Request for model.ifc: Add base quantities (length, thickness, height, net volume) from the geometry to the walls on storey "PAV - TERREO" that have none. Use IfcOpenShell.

First a look at what the model holds.

```python
import ifcopenshell
import ifcopenshell.util.element
import ifcopenshell.util.unit

model = ifcopenshell.open("model.ifc")
print(model.schema)
for unit_type in ("LENGTHUNIT", "AREAUNIT", "VOLUMEUNIT"):
    print(unit_type, ifcopenshell.util.unit.calculate_unit_scale(model, unit_type))
storey = next(s for s in model.by_type("IfcBuildingStorey") if s.Name == "PAV - TERREO")
walls = [e for e in ifcopenshell.util.element.get_decomposition(storey) if e.is_a("IfcWall")]
for e in sorted(walls, key=lambda e: e.id()):
    print(e.id(), e.is_a(), e.Name, list(ifcopenshell.util.element.get_psets(e, qtos_only=True)), sep=" | ")
```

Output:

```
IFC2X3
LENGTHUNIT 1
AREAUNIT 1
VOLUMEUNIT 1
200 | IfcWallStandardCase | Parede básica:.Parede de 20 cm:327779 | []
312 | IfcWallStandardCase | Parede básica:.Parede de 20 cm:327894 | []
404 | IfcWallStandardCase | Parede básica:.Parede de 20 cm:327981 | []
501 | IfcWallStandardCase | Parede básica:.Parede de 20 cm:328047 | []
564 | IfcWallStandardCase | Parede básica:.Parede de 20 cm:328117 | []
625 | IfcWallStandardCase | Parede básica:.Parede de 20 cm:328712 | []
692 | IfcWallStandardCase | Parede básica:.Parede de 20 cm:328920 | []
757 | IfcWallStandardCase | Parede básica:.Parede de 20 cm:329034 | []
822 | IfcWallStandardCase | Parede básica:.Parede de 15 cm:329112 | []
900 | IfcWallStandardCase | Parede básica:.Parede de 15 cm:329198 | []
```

```python
import ifcopenshell
import ifcopenshell.api.pset
import ifcopenshell.geom
import ifcopenshell.util.element
import ifcopenshell.util.shape
import ifcopenshell.util.unit

model = ifcopenshell.open("model.ifc")
unit_scale = ifcopenshell.util.unit.calculate_unit_scale(model)
volume_scale = ifcopenshell.util.unit.calculate_unit_scale(model, "VOLUMEUNIT")
settings = ifcopenshell.geom.settings()

storey = next(s for s in model.by_type("IfcBuildingStorey") if s.Name == "PAV - TERREO")
walls = [e for e in ifcopenshell.util.element.get_decomposition(storey) if e.is_a("IfcWall")]

for e in sorted(walls, key=lambda e: e.id()):
    if ifcopenshell.util.element.get_psets(e, qtos_only=True, should_inherit=False):
        continue
    # Geometry comes back in metres, in the element's own axes.
    shape = ifcopenshell.geom.create_shape(settings, e)
    values = {
        "Length": ifcopenshell.util.shape.get_x(shape.geometry) / unit_scale,
        "Width": ifcopenshell.util.shape.get_y(shape.geometry) / unit_scale,
        "Height": ifcopenshell.util.shape.get_z(shape.geometry) / unit_scale,
        "NetVolume": ifcopenshell.util.shape.get_volume(shape.geometry) / volume_scale,
    }
    qto = ifcopenshell.api.pset.add_qto(model, product=e, name="BaseQuantities")
    ifcopenshell.api.pset.edit_qto(model, qto=qto, properties=values)
    print(e.id(), {k: round(v, 3) for k, v in values.items()})

model.write("model_edited.ifc")
```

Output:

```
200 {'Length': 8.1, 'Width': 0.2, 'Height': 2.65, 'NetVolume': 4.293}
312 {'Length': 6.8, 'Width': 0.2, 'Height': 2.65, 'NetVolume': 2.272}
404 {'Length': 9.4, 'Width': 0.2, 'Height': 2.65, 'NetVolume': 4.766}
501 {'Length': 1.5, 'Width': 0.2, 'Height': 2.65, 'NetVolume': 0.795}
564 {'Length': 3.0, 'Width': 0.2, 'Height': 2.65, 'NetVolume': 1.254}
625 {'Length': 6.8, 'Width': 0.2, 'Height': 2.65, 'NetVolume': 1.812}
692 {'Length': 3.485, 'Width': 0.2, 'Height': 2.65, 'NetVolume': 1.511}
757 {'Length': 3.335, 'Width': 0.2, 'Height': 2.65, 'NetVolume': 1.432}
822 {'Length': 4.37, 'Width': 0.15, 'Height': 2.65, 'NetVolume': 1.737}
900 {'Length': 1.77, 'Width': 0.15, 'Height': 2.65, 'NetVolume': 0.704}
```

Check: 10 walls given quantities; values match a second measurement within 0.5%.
